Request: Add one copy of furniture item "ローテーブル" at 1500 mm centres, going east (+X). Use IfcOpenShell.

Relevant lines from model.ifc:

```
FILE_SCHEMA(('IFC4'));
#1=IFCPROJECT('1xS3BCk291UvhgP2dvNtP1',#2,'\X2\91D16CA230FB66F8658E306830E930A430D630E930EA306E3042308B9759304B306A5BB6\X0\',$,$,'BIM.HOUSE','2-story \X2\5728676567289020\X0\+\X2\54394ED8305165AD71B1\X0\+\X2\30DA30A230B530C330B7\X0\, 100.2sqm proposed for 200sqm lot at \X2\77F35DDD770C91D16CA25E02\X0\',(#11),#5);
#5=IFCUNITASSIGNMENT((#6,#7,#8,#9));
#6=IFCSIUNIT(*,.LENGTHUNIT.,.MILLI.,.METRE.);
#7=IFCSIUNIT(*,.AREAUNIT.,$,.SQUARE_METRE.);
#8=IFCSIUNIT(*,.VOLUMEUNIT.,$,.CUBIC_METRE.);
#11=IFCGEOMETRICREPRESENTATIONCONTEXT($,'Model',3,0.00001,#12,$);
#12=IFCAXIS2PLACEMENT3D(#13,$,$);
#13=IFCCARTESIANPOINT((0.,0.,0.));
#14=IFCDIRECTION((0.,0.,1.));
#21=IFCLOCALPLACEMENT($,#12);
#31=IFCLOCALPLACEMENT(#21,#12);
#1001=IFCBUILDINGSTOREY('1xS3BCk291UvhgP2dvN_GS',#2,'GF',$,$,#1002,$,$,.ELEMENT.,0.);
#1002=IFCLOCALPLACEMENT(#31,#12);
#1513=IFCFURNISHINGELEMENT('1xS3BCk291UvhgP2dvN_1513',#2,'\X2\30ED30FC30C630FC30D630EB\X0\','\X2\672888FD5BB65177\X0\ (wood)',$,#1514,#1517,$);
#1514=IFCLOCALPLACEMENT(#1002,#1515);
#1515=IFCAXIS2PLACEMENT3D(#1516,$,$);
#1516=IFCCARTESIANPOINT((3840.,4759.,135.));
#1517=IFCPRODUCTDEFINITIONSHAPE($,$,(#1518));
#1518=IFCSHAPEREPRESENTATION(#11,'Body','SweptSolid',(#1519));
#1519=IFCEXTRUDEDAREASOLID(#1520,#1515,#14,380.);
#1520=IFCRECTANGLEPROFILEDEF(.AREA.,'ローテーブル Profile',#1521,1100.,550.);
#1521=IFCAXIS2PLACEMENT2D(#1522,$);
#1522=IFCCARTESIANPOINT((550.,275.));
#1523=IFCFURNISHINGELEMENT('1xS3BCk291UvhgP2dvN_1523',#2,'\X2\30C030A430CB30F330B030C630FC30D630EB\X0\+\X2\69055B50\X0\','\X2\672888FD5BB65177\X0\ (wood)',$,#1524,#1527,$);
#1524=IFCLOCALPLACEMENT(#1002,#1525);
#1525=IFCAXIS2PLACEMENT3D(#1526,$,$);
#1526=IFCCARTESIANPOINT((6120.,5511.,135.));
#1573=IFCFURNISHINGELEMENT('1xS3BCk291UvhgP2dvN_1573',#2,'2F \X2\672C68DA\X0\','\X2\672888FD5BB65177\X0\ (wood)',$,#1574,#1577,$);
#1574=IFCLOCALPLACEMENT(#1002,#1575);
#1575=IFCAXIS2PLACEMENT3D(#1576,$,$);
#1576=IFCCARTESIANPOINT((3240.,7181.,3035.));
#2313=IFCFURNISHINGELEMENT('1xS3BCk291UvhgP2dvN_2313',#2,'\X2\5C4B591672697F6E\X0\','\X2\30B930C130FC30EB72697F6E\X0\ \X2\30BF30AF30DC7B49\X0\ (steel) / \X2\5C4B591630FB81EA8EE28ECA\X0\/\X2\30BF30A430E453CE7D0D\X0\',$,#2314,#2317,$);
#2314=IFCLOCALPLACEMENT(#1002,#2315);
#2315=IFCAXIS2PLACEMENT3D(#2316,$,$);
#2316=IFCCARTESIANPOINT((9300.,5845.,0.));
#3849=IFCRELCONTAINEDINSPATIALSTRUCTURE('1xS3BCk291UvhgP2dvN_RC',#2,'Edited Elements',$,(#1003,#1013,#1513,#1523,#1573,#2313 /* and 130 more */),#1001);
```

```python
import numpy as np
import ifcopenshell
import ifcopenshell.api.geometry
import ifcopenshell.api.root
import ifcopenshell.util.element
import ifcopenshell.util.placement

model = ifcopenshell.open("model.ifc")


def reuse_history(source, copy):
    """copy_class also copies each property set's owner history, people and application; keep the originals."""
    for rel in copy.IsDefinedBy:
        if rel.is_a("IfcRelDefinesByProperties") and (history := rel.RelatingPropertyDefinition.OwnerHistory):
            rel.RelatingPropertyDefinition.OwnerHistory = source.OwnerHistory
            ifcopenshell.util.element.remove_deep2(model, history)


source = model.by_id(1513)
base = ifcopenshell.util.placement.get_local_placement(source.ObjectPlacement)
step = np.array([1.0, 0.0, 0.0]) * 1500.0

for i in range(1, 2):
    copy = ifcopenshell.api.root.copy_class(model, product=source)
    copy.Representation = ifcopenshell.util.element.copy_deep(
        model, source.Representation, exclude=["IfcGeometricRepresentationContext", "IfcRepresentationMap"]
    )
    reuse_history(source, copy)
    matrix = base.copy()
    matrix[:3, 3] += i * step
    print("added at", matrix[:3, 3].round(3) + 0.0)
    ifcopenshell.api.geometry.edit_object_placement(model, product=copy, matrix=matrix, is_si=False)

model.write("model_rev.ifc")
```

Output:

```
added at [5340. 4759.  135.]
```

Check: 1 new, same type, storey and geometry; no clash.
